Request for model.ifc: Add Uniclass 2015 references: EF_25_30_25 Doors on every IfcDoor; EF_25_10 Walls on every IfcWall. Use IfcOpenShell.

First a look at what the model holds.

```python
import ifcopenshell

model = ifcopenshell.open("model.ifc")
print(model.schema)
print("classifications:", [c.Name for c in model.by_type("IfcClassification")])
for ifc_class in ("IfcDoor", "IfcRoof", "IfcStair", "IfcWall", "IfcWindow"):
    print(ifc_class, len(model.by_type(ifc_class)))
```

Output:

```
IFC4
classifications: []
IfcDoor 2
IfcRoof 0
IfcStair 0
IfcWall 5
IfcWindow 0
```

```python
import ifcopenshell
import ifcopenshell.api.classification

model = ifcopenshell.open("model.ifc")

system = ifcopenshell.api.classification.add_classification(model, classification="Uniclass 2015")

codes = {
    "IfcDoor": ("EF_25_30_25", "Doors"),
    "IfcWall": ("EF_25_10", "Walls"),
}
for ifc_class, (code, name) in codes.items():
    products = model.by_type(ifc_class)
    ifcopenshell.api.classification.add_reference(
        model, products=products, classification=system, identification=code, name=name
    )
    print(code, len(products))

model.write("model_edited.ifc")
```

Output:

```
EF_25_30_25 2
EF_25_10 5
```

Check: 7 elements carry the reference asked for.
